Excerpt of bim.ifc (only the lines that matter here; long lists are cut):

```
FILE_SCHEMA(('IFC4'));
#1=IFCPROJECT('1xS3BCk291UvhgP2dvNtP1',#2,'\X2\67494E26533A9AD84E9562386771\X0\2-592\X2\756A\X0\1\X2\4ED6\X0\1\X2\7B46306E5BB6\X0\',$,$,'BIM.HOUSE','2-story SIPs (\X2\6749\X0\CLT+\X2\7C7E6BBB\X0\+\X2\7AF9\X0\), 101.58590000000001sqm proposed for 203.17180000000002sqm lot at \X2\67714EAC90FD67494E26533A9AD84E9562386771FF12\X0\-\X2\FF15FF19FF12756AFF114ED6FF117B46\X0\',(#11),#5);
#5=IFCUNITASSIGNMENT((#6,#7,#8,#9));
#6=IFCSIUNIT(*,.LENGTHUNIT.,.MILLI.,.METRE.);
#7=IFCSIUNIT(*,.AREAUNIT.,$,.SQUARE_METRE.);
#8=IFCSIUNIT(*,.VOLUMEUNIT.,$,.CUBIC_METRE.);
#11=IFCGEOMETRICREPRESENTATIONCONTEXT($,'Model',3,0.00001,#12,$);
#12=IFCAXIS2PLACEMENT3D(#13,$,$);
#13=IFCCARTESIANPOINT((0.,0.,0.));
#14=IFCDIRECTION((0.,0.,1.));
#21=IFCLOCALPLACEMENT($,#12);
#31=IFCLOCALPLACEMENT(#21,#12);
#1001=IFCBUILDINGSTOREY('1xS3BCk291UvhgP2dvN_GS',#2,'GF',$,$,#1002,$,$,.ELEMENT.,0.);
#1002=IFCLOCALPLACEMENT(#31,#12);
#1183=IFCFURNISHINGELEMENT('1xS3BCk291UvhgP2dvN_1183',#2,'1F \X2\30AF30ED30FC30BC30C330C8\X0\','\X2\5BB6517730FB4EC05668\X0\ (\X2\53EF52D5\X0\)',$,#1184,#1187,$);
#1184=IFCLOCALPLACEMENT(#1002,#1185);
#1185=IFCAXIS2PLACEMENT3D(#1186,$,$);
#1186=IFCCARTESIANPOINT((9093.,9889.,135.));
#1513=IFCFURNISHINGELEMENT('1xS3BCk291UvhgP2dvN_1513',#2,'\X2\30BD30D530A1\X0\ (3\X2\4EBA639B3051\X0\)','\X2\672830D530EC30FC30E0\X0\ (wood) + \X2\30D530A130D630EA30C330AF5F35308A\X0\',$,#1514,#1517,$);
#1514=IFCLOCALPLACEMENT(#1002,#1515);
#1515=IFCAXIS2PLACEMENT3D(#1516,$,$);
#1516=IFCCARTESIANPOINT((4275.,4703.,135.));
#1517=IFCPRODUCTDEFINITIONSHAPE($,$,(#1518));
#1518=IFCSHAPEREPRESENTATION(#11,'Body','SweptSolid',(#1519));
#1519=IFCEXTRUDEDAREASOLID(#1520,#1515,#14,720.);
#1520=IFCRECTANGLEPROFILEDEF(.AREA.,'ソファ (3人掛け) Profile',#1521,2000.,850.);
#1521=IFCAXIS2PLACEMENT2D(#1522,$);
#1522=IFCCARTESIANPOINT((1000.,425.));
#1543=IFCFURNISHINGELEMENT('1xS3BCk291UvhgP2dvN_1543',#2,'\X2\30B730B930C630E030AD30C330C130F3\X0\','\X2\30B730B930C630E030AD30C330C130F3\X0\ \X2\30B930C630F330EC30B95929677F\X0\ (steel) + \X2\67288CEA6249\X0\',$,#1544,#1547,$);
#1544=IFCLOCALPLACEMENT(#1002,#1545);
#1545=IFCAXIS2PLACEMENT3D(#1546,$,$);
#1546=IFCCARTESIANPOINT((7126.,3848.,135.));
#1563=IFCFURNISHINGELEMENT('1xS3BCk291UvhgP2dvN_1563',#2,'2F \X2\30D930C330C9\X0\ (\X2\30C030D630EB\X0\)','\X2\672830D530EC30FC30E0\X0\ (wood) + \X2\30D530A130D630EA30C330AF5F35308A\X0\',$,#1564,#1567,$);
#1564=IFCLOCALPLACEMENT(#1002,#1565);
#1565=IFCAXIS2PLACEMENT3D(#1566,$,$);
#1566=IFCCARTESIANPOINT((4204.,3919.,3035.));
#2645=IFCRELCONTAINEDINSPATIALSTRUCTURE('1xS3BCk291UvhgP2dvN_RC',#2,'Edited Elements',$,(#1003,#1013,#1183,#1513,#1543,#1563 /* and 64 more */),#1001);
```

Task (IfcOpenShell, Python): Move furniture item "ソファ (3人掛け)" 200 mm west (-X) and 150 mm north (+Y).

```python
import ifcopenshell
import ifcopenshell.api.geometry
import ifcopenshell.util.placement
import ifcopenshell.util.unit

model = ifcopenshell.open("bim.ifc")
unit_scale = ifcopenshell.util.unit.calculate_unit_scale(model)

item = model.by_id(1513)
matrix = ifcopenshell.util.placement.get_local_placement(item.ObjectPlacement)
matrix[0, 3] -= 0.2 / unit_scale
matrix[1, 3] += 0.15 / unit_scale
ifcopenshell.api.geometry.edit_object_placement(model, product=item, matrix=matrix, is_si=False)

print(ifcopenshell.util.placement.get_local_placement(item.ObjectPlacement).round(3) + 0.0)

model.write("bim-out.ifc")
```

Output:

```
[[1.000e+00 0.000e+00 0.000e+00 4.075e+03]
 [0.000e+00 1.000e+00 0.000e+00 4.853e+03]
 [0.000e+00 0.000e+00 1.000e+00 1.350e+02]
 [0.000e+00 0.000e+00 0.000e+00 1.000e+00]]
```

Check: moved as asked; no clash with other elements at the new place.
